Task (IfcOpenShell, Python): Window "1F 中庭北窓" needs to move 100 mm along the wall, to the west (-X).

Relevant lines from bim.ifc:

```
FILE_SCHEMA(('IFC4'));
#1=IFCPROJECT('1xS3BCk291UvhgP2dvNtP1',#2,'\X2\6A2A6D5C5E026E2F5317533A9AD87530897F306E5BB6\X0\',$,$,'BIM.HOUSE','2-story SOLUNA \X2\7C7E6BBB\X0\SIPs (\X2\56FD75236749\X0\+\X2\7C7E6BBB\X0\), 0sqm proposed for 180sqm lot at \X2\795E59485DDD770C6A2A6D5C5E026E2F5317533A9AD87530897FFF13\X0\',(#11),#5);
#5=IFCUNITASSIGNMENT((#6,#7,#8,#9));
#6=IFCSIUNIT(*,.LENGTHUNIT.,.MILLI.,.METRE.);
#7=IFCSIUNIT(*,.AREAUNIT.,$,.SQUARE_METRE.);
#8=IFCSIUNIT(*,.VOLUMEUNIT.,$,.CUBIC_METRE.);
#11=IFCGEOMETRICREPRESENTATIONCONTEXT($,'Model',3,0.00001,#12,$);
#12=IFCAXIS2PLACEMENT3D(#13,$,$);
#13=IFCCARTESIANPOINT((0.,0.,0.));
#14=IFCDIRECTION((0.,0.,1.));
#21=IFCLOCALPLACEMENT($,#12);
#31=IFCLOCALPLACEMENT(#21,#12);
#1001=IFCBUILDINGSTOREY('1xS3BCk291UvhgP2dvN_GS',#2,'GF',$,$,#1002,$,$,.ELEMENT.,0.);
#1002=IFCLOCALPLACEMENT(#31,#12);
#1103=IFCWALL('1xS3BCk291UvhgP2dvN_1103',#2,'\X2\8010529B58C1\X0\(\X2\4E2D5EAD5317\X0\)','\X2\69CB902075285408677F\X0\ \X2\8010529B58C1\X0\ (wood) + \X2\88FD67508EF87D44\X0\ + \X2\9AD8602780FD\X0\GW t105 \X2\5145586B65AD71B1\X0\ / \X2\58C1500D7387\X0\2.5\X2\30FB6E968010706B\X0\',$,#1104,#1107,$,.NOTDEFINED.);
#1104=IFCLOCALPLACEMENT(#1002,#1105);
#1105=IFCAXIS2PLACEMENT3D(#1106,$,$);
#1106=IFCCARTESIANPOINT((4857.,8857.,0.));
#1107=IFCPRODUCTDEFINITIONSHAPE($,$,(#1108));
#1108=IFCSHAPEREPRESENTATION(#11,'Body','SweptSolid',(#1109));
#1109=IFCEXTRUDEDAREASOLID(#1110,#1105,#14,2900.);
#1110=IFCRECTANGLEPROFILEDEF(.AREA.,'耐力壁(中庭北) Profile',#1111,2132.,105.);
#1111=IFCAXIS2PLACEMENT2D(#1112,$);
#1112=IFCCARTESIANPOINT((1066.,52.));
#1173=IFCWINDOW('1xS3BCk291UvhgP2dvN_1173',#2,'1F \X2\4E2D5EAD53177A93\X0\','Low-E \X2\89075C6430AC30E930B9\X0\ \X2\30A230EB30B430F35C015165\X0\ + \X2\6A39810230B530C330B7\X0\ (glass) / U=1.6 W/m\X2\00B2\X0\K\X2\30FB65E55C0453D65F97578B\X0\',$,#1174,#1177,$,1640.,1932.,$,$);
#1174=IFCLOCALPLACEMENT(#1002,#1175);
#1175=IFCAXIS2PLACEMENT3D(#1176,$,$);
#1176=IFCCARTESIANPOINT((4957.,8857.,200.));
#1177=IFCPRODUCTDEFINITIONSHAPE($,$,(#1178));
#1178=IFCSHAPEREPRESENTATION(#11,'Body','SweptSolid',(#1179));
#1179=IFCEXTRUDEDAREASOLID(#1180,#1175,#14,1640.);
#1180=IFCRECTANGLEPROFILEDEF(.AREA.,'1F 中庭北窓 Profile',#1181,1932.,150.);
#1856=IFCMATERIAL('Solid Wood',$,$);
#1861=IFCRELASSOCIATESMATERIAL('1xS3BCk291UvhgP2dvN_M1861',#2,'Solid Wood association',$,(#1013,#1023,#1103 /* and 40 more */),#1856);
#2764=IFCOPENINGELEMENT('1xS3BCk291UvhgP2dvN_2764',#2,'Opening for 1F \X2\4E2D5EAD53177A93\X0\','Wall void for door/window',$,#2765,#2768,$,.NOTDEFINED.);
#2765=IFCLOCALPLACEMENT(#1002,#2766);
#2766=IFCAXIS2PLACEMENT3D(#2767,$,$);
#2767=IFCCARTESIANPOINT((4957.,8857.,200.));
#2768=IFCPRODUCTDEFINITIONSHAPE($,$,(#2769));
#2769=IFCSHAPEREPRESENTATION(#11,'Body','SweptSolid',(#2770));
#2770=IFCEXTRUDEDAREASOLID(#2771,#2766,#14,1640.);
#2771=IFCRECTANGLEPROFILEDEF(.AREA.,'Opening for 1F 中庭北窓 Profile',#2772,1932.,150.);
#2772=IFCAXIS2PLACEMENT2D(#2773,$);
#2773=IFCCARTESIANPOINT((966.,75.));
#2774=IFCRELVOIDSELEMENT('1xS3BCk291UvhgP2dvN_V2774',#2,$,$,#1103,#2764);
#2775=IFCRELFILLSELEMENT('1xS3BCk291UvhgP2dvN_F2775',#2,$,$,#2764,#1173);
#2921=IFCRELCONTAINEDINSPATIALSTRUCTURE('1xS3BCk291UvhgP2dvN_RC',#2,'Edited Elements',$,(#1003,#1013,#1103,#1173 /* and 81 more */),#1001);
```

```python
import ifcopenshell
import ifcopenshell.api.geometry
import ifcopenshell.util.placement
import ifcopenshell.util.unit

model = ifcopenshell.open("bim.ifc")
unit_scale = ifcopenshell.util.unit.calculate_unit_scale(model)

window = model.by_id(1173)
opening = window.FillsVoids[0].RelatingOpeningElement
wall = opening.VoidsElements[0].RelatingBuildingElement

wall_matrix = ifcopenshell.util.placement.get_local_placement(wall.ObjectPlacement)
shift = wall_matrix[:3, 0] * -0.1 / unit_scale
before = ifcopenshell.util.placement.get_local_placement(window.ObjectPlacement)[:3, 3].copy()

# The window is not placed relative to its opening, so move both.
for product in (opening, window):
    matrix = ifcopenshell.util.placement.get_local_placement(product.ObjectPlacement)
    matrix[:3, 3] += shift
    ifcopenshell.api.geometry.edit_object_placement(model, product=product, matrix=matrix, is_si=False)

after = ifcopenshell.util.placement.get_local_placement(window.ObjectPlacement)[:3, 3]
print("window moved by", (after - before).round(3) + 0.0)

model.write("bim_rev.ifc")
```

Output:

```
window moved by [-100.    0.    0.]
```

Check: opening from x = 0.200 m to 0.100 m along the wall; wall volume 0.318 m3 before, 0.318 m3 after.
